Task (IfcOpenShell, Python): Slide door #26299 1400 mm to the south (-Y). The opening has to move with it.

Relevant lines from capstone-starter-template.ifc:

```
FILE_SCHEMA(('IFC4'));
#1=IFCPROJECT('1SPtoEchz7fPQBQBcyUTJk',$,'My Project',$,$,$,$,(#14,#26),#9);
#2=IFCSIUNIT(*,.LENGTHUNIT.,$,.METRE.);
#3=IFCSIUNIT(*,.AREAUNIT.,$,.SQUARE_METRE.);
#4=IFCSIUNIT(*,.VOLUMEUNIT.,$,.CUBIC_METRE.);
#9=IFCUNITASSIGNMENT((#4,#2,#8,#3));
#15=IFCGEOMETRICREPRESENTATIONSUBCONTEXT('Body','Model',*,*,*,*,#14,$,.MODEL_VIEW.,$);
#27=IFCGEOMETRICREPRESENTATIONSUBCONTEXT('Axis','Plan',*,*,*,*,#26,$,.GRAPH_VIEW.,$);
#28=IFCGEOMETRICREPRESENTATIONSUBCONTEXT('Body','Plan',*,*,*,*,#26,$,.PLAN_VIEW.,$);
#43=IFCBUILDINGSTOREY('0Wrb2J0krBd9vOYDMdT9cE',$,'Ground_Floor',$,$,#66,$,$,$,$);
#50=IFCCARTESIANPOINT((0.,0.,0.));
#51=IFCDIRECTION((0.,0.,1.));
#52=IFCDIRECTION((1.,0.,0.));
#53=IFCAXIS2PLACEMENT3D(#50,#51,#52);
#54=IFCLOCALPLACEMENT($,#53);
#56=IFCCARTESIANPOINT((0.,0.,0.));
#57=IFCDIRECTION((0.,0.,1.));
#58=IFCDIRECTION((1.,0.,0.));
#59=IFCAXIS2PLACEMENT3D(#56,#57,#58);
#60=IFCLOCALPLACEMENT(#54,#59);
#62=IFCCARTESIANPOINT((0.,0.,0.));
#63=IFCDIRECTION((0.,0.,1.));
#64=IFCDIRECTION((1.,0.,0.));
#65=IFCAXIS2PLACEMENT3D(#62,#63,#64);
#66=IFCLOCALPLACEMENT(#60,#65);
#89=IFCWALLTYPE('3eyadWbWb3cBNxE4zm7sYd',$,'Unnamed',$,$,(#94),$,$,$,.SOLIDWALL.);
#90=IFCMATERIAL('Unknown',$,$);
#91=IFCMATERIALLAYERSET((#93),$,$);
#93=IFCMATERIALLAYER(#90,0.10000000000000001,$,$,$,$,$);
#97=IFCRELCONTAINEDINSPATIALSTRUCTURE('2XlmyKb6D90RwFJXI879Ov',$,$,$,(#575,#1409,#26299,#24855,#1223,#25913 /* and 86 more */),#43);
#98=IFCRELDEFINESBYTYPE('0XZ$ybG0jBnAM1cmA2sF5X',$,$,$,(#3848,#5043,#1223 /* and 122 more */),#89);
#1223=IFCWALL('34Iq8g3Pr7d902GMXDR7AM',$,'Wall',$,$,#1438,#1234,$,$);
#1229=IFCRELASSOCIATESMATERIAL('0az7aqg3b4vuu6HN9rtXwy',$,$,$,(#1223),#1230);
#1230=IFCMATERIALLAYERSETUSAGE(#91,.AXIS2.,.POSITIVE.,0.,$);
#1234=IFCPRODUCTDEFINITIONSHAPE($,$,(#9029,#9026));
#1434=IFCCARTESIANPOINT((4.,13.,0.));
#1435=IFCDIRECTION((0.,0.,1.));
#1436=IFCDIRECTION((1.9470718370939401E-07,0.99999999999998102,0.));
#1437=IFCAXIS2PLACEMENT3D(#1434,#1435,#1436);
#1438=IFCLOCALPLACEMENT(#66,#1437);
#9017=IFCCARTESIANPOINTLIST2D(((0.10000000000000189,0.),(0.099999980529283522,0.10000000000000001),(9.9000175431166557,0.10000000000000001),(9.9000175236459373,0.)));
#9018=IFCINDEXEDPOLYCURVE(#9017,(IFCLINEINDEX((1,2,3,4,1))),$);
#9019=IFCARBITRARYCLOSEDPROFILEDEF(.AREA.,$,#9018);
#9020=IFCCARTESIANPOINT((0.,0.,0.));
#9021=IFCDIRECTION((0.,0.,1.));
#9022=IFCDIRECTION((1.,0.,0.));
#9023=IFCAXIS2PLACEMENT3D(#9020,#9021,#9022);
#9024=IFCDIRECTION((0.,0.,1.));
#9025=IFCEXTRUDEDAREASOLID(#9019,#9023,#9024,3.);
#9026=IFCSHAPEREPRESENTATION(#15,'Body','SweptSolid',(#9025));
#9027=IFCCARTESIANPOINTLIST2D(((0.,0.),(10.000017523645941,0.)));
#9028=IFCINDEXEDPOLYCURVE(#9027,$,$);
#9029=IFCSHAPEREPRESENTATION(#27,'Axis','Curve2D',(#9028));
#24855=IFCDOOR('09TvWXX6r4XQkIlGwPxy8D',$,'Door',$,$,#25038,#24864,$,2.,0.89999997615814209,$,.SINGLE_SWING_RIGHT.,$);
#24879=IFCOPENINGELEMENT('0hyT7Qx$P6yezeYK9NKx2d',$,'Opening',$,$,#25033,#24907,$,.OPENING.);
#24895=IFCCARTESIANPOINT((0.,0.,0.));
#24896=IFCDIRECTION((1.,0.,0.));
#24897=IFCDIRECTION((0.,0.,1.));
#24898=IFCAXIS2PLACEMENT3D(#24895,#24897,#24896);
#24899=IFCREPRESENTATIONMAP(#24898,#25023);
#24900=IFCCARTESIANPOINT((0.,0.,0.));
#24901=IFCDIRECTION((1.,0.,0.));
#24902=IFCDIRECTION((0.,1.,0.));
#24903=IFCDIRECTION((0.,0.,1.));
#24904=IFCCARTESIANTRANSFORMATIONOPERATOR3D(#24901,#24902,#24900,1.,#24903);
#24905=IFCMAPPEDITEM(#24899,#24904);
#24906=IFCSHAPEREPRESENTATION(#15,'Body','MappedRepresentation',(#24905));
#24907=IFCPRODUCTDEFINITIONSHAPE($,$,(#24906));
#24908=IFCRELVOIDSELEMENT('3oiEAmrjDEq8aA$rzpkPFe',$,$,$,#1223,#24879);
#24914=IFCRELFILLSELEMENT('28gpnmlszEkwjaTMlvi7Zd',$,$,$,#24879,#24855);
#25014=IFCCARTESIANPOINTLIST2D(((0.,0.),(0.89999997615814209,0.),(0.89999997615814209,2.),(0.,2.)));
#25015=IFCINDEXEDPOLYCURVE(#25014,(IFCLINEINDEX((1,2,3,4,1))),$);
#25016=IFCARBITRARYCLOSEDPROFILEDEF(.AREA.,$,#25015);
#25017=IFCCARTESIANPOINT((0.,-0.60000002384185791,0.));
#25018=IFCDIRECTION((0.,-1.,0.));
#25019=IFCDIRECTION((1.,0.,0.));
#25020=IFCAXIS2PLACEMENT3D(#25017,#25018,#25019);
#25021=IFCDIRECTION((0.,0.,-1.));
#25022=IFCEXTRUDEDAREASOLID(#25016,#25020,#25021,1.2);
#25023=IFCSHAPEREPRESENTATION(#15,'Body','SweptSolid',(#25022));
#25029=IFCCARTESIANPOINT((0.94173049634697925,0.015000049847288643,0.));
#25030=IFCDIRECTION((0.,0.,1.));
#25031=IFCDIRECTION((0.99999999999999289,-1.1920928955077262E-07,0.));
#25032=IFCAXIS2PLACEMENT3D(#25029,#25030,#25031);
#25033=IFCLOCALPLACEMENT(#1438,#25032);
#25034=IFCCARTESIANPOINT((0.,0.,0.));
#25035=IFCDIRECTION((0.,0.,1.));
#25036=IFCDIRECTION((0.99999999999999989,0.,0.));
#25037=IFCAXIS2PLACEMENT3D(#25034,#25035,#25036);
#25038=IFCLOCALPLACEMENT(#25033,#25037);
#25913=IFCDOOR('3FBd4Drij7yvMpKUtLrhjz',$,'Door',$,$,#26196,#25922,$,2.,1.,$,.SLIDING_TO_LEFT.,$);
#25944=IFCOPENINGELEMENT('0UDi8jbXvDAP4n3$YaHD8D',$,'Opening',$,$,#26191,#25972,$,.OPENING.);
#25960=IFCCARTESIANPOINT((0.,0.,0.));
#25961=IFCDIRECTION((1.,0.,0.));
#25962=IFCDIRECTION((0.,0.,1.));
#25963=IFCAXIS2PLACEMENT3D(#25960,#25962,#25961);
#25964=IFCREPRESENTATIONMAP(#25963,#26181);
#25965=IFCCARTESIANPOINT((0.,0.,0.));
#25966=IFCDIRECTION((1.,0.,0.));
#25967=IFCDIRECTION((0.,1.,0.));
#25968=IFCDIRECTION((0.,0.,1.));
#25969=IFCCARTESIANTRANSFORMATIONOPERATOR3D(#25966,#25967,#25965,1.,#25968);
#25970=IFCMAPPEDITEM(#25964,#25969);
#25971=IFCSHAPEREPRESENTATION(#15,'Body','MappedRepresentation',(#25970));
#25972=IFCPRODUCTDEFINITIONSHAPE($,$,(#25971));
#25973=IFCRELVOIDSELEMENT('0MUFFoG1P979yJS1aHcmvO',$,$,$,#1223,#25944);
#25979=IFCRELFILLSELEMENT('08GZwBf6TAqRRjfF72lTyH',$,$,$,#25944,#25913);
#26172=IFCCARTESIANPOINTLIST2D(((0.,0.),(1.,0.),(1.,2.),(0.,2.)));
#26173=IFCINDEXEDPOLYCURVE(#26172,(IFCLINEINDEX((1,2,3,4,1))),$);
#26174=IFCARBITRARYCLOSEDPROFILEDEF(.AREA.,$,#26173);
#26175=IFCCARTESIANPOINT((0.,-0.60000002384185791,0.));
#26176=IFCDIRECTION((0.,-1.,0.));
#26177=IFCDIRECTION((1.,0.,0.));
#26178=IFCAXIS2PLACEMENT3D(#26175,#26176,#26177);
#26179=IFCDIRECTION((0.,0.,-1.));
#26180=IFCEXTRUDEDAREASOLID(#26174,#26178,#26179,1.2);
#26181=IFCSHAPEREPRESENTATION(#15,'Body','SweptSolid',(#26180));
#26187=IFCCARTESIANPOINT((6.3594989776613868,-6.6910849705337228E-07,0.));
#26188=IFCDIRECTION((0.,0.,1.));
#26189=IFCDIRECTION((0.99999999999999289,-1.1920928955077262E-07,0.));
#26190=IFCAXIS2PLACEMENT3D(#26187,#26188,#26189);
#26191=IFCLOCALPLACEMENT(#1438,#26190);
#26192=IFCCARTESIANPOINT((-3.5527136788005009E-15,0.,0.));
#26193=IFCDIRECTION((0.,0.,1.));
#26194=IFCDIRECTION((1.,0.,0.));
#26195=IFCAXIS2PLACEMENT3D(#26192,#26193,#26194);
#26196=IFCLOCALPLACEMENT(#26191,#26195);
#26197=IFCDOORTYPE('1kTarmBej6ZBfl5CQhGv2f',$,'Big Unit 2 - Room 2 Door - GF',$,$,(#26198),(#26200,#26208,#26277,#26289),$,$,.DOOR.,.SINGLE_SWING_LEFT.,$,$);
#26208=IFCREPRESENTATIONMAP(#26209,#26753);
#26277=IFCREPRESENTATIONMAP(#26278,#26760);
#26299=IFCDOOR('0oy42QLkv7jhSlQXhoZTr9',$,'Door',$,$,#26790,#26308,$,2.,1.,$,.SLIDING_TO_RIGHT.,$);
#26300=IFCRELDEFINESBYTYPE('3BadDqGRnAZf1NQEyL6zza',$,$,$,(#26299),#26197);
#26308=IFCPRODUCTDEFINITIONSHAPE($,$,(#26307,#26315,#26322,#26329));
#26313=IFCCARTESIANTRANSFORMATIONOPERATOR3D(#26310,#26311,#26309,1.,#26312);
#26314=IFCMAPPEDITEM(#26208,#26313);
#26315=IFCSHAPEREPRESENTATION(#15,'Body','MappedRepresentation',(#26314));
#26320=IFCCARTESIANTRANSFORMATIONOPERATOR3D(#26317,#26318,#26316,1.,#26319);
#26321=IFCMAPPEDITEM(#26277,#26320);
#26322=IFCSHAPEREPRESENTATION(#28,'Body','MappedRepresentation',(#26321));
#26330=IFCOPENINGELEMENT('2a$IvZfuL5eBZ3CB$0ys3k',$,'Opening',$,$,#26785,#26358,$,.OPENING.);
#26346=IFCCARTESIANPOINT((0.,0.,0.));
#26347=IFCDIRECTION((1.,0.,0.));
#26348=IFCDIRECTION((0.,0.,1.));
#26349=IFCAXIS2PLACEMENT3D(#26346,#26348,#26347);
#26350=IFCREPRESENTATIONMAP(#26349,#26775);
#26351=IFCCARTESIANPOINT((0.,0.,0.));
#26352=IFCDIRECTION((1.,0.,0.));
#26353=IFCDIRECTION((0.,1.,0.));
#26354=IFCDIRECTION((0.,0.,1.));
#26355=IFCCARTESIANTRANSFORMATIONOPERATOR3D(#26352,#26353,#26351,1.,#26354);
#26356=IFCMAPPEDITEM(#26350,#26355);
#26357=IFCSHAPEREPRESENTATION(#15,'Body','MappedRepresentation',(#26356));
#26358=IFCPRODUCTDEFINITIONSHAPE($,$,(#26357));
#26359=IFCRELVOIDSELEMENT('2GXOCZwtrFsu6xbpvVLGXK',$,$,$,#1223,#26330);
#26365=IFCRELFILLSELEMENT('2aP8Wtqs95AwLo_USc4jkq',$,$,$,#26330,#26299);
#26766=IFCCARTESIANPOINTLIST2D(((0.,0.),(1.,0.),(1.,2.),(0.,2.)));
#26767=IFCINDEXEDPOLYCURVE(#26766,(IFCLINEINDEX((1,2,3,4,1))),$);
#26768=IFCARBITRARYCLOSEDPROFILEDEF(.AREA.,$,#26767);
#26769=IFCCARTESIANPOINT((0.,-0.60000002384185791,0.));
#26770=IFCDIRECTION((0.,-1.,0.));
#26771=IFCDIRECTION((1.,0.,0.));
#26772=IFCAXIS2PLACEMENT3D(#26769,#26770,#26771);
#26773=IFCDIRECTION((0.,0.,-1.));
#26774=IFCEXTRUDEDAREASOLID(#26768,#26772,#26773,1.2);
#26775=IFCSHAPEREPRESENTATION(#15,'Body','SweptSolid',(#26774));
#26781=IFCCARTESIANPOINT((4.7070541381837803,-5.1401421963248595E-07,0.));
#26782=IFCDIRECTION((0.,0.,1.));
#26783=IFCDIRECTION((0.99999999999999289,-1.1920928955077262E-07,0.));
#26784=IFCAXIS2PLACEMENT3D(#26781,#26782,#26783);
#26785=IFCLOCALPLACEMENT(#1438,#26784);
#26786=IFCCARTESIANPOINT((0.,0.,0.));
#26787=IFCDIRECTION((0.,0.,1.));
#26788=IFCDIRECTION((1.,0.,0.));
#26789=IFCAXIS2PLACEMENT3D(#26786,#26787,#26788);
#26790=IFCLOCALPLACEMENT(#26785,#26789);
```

```python
import ifcopenshell
import ifcopenshell.api.geometry
import ifcopenshell.util.placement
import ifcopenshell.util.unit

model = ifcopenshell.open("capstone-starter-template.ifc")
unit_scale = ifcopenshell.util.unit.calculate_unit_scale(model)

door = model.by_guid("0oy42QLkv7jhSlQXhoZTr9")
opening = door.FillsVoids[0].RelatingOpeningElement
wall = opening.VoidsElements[0].RelatingBuildingElement

wall_matrix = ifcopenshell.util.placement.get_local_placement(wall.ObjectPlacement)
shift = wall_matrix[:3, 0] * -1.4 / unit_scale
before = ifcopenshell.util.placement.get_local_placement(door.ObjectPlacement)[:3, 3].copy()

# The door is placed relative to its opening, so it follows when the opening moves.
matrix = ifcopenshell.util.placement.get_local_placement(opening.ObjectPlacement)
matrix[:3, 3] += shift
ifcopenshell.api.geometry.edit_object_placement(
    model, product=opening, matrix=matrix, is_si=False, should_transform_children=True
)

after = ifcopenshell.util.placement.get_local_placement(door.ObjectPlacement)[:3, 3]
print("door moved by", (after - before).round(3) + 0.0)

model.write("capstone-starter-template_edited.ifc")
```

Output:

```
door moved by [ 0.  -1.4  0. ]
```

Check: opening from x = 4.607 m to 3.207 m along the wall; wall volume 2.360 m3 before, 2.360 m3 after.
